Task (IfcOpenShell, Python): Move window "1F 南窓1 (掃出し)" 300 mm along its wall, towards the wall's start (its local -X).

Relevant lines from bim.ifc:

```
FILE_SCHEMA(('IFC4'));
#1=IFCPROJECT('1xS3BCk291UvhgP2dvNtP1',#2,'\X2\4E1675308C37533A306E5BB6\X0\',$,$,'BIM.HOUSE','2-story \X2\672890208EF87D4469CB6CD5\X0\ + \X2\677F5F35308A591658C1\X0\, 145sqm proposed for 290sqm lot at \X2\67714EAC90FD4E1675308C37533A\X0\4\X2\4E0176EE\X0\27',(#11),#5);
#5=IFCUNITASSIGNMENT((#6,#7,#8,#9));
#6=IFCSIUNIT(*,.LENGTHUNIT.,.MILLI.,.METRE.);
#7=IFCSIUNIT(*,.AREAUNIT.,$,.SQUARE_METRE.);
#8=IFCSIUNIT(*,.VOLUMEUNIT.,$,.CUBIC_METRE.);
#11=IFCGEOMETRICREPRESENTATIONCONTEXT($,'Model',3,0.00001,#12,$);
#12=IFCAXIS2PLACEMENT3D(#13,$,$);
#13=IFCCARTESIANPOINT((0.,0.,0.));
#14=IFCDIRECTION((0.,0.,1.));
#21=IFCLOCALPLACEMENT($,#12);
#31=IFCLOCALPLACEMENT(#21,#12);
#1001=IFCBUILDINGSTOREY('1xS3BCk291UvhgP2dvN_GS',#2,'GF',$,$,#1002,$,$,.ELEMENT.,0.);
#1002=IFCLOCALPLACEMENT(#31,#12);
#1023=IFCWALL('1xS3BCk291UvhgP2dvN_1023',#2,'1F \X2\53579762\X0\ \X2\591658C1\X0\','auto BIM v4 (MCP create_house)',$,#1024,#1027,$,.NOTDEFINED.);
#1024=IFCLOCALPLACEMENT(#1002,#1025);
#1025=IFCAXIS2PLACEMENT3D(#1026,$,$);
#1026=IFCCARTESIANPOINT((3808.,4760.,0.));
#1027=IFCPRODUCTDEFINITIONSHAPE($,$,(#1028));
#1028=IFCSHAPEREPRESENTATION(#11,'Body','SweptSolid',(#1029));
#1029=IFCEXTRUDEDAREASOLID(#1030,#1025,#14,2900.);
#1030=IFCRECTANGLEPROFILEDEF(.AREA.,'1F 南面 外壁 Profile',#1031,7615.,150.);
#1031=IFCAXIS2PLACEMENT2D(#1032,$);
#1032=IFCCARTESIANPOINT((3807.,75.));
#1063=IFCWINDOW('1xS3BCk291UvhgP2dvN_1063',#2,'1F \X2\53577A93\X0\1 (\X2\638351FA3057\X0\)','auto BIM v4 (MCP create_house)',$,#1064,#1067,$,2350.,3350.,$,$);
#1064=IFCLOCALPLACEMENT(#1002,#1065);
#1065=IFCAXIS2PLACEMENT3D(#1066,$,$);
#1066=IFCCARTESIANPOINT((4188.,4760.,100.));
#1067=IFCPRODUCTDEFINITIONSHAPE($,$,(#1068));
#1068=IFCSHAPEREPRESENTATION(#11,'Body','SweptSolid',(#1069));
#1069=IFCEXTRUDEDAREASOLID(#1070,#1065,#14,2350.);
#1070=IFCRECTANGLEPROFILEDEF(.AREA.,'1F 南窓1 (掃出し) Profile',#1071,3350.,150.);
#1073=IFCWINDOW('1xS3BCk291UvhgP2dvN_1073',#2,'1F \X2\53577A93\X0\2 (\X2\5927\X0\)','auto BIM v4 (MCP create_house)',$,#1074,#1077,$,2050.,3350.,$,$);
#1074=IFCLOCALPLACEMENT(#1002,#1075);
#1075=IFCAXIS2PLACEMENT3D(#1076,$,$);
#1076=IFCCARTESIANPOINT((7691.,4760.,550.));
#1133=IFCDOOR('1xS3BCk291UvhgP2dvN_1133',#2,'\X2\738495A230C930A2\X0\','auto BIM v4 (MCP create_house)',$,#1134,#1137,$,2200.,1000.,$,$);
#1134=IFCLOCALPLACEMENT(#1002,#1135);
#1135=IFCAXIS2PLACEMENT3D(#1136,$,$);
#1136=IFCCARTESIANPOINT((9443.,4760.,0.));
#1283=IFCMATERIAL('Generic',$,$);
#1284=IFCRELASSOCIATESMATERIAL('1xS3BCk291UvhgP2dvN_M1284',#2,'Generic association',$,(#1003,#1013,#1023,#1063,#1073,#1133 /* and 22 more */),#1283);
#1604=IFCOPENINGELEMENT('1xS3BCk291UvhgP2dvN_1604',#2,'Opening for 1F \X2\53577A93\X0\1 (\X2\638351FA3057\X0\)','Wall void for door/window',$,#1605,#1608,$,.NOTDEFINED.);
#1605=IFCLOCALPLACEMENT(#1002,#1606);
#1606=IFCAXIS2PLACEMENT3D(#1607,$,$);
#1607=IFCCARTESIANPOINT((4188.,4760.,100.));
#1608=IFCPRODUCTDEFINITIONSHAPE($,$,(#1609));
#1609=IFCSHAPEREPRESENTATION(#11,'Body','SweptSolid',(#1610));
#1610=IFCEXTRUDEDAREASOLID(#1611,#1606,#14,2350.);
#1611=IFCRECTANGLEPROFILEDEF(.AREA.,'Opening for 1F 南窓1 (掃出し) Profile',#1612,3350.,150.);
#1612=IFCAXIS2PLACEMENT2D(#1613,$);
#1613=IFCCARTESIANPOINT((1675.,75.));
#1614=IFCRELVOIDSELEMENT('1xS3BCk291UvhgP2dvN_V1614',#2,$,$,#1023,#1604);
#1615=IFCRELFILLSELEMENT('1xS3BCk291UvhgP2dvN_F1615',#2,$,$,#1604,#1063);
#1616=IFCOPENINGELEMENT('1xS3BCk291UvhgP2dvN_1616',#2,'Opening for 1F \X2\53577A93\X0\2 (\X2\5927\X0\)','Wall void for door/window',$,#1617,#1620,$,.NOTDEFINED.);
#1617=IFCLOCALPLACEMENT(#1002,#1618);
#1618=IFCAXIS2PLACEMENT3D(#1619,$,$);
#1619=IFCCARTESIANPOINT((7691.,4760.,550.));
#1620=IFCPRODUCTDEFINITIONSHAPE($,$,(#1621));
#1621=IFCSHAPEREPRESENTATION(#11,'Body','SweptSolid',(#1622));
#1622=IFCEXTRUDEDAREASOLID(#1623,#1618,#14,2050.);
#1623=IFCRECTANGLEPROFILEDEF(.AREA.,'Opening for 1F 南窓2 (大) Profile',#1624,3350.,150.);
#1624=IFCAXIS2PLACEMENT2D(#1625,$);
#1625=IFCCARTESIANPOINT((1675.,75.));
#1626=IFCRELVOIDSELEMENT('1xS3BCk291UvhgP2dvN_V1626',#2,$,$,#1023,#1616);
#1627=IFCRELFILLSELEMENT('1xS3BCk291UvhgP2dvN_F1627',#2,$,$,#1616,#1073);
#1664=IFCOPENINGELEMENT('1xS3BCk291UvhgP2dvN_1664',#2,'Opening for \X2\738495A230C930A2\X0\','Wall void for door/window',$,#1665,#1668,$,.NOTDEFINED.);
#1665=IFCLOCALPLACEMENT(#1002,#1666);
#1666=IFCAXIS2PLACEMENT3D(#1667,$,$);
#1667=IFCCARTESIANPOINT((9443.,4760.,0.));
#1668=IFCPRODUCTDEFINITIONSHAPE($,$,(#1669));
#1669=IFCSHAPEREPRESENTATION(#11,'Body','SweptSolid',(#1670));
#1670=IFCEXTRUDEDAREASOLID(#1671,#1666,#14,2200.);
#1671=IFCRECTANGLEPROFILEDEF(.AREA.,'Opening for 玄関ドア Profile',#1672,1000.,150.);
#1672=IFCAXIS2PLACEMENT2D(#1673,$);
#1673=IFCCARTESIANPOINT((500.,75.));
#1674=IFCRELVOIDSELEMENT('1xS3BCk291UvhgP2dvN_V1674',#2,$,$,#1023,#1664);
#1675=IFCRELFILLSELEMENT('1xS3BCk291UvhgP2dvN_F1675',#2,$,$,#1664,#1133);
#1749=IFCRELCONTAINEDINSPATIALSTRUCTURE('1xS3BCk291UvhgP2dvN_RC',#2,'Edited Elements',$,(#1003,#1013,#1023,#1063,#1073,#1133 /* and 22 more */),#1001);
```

```python
import ifcopenshell
import ifcopenshell.api.geometry
import ifcopenshell.util.placement

model = ifcopenshell.open("bim.ifc")

window = model.by_id(1063)
opening = window.FillsVoids[0].RelatingOpeningElement
wall = opening.VoidsElements[0].RelatingBuildingElement

wall_matrix = ifcopenshell.util.placement.get_local_placement(wall.ObjectPlacement)
shift = wall_matrix[:3, 0] * -300.0
before = ifcopenshell.util.placement.get_local_placement(window.ObjectPlacement)[:3, 3].copy()

# The window is not placed relative to its opening, so move both.
for product in (opening, window):
    matrix = ifcopenshell.util.placement.get_local_placement(product.ObjectPlacement)
    matrix[:3, 3] += shift
    ifcopenshell.api.geometry.edit_object_placement(model, product=product, matrix=matrix, is_si=False)

after = ifcopenshell.util.placement.get_local_placement(window.ObjectPlacement)[:3, 3]
print("window moved by", (after - before).round(3) + 0.0)

model.write("bim_v2.ifc")
```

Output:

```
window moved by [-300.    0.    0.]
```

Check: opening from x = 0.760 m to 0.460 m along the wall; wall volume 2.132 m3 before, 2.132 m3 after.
